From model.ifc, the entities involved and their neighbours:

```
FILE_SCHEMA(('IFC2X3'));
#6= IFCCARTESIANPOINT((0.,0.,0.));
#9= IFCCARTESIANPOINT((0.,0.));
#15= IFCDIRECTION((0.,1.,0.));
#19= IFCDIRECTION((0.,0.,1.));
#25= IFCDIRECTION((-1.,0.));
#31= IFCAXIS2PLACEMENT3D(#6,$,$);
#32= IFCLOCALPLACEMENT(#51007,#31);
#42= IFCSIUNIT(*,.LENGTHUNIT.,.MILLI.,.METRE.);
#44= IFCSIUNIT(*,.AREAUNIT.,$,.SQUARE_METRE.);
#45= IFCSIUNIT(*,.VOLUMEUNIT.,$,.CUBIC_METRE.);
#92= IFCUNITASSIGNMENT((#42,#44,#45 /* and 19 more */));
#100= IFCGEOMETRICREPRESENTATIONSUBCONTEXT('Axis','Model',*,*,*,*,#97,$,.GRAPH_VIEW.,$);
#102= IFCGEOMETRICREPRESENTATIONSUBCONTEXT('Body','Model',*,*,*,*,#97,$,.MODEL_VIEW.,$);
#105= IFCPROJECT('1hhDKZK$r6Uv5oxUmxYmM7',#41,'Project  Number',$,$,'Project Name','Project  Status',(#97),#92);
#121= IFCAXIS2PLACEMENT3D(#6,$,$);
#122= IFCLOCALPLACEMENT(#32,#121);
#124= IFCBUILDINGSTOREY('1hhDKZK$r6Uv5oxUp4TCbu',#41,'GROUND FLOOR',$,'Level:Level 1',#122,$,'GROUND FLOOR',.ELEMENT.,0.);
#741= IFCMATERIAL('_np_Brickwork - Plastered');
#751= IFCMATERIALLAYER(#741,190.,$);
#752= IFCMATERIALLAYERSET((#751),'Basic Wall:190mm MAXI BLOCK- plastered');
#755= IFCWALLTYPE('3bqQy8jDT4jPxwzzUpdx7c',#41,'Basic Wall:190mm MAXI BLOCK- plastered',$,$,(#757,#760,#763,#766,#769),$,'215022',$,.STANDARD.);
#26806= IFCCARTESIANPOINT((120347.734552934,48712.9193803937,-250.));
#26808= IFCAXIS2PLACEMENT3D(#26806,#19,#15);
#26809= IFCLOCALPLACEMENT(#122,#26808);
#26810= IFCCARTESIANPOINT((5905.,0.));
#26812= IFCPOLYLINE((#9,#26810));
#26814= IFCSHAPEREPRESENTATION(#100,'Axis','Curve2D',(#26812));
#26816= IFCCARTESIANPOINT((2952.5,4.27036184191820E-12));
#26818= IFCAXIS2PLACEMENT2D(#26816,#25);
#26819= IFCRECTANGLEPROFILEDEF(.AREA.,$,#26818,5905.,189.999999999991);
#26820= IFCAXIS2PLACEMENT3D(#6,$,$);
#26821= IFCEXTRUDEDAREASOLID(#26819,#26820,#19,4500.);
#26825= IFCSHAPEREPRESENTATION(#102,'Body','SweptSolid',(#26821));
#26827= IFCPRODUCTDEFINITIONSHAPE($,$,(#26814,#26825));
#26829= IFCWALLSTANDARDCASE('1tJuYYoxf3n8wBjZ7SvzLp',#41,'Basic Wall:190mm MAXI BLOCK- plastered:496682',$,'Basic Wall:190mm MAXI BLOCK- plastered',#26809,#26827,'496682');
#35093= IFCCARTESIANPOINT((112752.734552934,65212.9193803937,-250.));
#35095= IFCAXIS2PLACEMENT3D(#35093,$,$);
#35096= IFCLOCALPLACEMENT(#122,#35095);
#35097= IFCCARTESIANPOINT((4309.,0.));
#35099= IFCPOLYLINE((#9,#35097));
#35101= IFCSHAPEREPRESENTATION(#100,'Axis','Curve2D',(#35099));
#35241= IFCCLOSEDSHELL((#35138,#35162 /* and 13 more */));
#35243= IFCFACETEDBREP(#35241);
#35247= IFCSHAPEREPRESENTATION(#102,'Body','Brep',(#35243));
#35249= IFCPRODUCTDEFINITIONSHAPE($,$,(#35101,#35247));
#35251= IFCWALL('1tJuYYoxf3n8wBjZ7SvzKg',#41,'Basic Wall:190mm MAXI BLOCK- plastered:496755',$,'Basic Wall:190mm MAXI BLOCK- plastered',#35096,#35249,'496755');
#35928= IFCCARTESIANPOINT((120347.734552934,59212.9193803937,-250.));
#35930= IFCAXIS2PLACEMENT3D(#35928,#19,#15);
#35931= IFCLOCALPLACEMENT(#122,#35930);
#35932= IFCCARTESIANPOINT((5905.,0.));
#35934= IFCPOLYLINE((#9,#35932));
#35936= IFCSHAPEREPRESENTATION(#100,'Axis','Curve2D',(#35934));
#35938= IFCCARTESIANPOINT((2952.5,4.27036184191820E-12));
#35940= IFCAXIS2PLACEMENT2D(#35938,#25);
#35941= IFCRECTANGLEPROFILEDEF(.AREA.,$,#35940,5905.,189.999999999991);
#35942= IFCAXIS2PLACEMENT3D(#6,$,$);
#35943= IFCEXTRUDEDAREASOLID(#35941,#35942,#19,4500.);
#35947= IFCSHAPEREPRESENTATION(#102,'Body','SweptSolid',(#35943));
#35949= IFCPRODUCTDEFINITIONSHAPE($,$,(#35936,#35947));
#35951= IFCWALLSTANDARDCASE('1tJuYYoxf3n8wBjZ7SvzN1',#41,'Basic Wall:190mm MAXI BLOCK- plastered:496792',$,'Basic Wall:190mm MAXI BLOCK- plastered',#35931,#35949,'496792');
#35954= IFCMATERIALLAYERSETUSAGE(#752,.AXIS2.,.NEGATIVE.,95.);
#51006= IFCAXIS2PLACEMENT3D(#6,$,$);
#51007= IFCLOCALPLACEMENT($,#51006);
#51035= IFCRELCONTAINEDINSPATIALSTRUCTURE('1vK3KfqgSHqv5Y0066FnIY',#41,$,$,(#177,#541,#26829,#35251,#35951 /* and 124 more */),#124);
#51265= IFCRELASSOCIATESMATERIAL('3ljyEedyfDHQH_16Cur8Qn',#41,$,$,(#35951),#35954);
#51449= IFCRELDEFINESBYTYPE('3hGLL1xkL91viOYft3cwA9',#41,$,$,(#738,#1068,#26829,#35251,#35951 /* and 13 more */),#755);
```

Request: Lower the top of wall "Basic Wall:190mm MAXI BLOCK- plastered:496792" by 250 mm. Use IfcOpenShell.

```python
import ifcopenshell
import ifcopenshell.geom
import ifcopenshell.util.representation
import ifcopenshell.util.shape

model = ifcopenshell.open("model.ifc")
settings = ifcopenshell.geom.settings()


def volume(element):
    """Net volume in cubic metres, openings subtracted."""
    shape = ifcopenshell.geom.create_shape(settings, element)
    return ifcopenshell.util.shape.get_volume(shape.geometry)


wall = model.by_guid("1tJuYYoxf3n8wBjZ7SvzN1")
before = volume(wall)

body = ifcopenshell.util.representation.get_representation(wall, "Model", "Body")
solid = body.Items[0]
old_height = solid.Depth
solid.Depth -= 250.0
after = volume(wall)

print(f"height {old_height:g} -> {solid.Depth:g}, volume {before:.3f} -> {after:.3f} m3")

model.write("model_rev.ifc")
```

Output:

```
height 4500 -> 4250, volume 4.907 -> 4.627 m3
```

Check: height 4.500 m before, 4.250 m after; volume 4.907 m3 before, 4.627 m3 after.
